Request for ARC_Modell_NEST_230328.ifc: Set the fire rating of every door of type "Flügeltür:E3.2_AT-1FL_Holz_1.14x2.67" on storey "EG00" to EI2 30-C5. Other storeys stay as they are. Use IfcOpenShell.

First a look at what the model holds.

```python
import ifcopenshell
import ifcopenshell.util.element

model = ifcopenshell.open("ARC_Modell_NEST_230328.ifc")
print(model.schema)
storey = next(s for s in model.by_type("IfcBuildingStorey") if s.Name == "EG00")
doors = [e for e in ifcopenshell.util.element.get_decomposition(storey) if e.is_a("IfcDoor")]
seen = {}
for e in doors:
    element_type = ifcopenshell.util.element.get_type(e)
    key = (element_type.Name if element_type != e and element_type else None, ifcopenshell.util.element.get_pset(e, "Pset_DoorCommon", "FireRating"))
    seen[key] = seen.get(key, 0) + 1
for (name, value), count in sorted(seen.items(), key=str):
    print(count, "x", name, "|", value)
```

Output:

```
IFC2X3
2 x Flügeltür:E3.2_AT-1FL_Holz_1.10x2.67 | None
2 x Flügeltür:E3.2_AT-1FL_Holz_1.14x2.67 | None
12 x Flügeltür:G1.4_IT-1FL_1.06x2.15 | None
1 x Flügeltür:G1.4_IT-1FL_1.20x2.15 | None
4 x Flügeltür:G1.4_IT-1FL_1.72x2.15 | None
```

```python
import ifcopenshell
import ifcopenshell.api.pset
import ifcopenshell.util.element

model = ifcopenshell.open("ARC_Modell_NEST_230328.ifc")

storey = next(s for s in model.by_type("IfcBuildingStorey") if s.Name == "EG00")
doors = [e for e in ifcopenshell.util.element.get_decomposition(storey) if e.is_a("IfcDoor")]

count = 0
for e in doors:
    element_type = ifcopenshell.util.element.get_type(e)
    if element_type in (None, e) or element_type.Name != "Flügeltür:E3.2_AT-1FL_Holz_1.14x2.67":
        continue
    # add_pset returns the element's existing set when there is one.
    pset = ifcopenshell.api.pset.add_pset(model, product=e, name="Pset_DoorCommon")
    ifcopenshell.api.pset.edit_pset(model, pset=pset, properties={"FireRating": "EI2 30-C5"})
    count += 1

print(count, "doors updated")

model.write("ARC_Modell_NEST_230328_v2.ifc")
```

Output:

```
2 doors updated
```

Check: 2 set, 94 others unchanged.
